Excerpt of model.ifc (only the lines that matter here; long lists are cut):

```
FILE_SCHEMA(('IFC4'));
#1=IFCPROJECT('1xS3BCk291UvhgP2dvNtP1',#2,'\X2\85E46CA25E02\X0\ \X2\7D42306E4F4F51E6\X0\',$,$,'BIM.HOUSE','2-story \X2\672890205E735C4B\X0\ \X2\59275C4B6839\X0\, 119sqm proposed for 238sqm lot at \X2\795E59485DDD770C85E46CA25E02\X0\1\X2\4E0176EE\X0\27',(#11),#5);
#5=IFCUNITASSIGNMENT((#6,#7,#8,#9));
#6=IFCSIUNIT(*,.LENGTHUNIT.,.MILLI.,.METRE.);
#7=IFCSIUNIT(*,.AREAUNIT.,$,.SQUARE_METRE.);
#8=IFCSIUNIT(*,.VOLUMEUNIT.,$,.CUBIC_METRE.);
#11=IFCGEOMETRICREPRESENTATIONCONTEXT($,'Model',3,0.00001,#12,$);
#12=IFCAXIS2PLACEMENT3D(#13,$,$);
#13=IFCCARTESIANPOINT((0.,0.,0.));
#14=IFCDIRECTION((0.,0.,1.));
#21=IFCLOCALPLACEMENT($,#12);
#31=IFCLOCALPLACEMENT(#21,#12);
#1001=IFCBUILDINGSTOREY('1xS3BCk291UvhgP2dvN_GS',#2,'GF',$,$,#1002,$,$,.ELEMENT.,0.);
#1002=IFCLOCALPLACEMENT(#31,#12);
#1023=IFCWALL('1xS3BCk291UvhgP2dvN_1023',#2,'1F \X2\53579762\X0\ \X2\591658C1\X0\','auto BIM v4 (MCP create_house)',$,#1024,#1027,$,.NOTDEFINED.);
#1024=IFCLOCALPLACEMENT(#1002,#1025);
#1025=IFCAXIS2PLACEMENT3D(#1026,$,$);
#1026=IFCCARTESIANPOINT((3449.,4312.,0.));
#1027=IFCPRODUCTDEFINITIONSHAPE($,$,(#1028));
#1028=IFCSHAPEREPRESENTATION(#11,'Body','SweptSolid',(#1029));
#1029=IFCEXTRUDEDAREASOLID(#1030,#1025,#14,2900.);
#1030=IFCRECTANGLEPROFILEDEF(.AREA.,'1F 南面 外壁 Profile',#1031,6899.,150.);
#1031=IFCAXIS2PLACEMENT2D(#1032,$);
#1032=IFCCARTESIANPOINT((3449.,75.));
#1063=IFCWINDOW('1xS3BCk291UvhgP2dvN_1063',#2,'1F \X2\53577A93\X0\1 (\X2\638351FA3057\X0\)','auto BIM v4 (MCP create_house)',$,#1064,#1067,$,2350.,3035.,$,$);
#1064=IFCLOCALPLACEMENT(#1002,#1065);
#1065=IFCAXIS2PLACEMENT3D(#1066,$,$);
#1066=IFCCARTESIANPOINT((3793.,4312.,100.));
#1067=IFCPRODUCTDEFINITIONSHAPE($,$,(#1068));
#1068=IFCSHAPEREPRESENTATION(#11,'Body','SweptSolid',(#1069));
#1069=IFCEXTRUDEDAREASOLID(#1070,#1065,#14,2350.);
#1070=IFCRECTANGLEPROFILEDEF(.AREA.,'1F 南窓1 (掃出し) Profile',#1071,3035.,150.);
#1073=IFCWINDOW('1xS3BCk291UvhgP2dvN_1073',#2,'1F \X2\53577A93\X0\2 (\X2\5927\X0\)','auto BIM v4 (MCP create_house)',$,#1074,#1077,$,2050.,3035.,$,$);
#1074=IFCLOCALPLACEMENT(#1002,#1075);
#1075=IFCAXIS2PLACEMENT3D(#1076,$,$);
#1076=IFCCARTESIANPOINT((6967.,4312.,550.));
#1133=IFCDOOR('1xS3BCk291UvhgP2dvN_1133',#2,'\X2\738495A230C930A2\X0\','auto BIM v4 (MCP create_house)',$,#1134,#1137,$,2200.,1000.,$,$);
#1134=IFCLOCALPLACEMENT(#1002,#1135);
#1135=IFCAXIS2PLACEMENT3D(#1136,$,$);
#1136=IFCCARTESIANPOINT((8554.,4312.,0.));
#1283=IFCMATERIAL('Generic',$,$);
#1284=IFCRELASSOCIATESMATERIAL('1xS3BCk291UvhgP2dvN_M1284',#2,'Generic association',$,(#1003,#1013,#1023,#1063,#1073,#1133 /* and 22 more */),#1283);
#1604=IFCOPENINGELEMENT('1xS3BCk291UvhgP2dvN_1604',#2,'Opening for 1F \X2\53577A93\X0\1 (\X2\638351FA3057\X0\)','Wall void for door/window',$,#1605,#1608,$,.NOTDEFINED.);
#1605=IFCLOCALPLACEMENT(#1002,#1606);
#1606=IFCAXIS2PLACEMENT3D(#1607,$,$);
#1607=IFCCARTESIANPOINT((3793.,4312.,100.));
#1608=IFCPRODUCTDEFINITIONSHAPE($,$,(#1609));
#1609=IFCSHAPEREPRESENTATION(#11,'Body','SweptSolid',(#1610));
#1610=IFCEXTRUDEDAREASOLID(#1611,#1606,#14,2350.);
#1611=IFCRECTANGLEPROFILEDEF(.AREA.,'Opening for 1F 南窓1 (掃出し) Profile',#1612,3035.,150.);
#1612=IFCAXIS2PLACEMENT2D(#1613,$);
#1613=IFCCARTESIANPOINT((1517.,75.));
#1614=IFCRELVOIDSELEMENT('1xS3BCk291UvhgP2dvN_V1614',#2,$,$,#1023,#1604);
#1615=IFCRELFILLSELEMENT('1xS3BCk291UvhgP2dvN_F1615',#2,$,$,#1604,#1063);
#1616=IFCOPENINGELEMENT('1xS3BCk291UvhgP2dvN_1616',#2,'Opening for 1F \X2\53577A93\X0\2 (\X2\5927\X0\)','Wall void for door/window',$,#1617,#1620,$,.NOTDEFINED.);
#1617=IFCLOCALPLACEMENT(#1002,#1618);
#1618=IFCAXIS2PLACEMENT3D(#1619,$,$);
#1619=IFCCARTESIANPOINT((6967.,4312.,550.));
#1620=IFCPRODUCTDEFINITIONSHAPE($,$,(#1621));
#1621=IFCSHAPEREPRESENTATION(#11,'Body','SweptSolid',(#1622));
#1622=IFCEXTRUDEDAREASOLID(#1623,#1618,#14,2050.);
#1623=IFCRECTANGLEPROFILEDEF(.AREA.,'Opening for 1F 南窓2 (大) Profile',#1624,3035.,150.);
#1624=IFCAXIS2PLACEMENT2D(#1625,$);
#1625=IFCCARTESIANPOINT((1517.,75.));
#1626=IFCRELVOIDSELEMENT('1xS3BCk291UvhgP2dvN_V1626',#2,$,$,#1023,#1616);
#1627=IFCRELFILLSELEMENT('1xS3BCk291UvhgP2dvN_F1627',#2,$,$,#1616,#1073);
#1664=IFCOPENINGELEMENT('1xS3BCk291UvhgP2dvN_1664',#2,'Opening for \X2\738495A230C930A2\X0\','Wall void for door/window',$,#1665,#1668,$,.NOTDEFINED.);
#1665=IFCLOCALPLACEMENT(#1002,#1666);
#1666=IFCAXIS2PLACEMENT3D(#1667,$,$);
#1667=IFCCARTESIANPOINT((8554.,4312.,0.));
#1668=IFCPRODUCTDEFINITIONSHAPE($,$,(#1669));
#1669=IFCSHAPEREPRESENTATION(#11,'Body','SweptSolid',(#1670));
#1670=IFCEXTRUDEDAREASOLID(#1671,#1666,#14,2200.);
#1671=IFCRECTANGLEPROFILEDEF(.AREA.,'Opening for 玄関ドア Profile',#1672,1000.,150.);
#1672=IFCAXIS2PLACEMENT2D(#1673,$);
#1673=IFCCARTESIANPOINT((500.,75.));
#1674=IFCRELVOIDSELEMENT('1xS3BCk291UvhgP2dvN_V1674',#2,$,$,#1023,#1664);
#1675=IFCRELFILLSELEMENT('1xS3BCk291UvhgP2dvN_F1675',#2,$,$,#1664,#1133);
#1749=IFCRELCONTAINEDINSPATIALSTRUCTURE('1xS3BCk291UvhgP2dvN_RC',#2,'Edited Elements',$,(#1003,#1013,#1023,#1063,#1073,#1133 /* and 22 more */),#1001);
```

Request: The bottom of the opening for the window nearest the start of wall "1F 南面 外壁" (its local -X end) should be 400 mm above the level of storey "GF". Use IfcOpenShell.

```python
import numpy as np
import ifcopenshell
import ifcopenshell.api.geometry
import ifcopenshell.geom
import ifcopenshell.util.element
import ifcopenshell.util.placement
import ifcopenshell.util.shape
import ifcopenshell.util.unit

model = ifcopenshell.open("model.ifc")
unit_scale = ifcopenshell.util.unit.calculate_unit_scale(model)

window = model.by_id(1063)
opening = window.FillsVoids[0].RelatingOpeningElement
storey = ifcopenshell.util.element.get_container(window, ifc_class="IfcBuildingStorey")
level = ifcopenshell.util.placement.get_local_placement(storey.ObjectPlacement)[2, 3]

# The opening's origin need not be at the sill, so measure its lowest point.
shape = ifcopenshell.geom.create_shape(ifcopenshell.geom.settings(), opening)
bottom = ifcopenshell.util.shape.get_shape_bottom_elevation(shape, shape.geometry) / unit_scale
dz = level + 400.0 - bottom

shift = np.array([0.0, 0.0, dz])
# The window is not placed relative to its opening, so move both.
for product in (opening, window):
    matrix = ifcopenshell.util.placement.get_local_placement(product.ObjectPlacement)
    matrix[:3, 3] += shift
    ifcopenshell.api.geometry.edit_object_placement(model, product=product, matrix=matrix, is_si=False)

print(f"moved by {dz * unit_scale:+.3f} m")

model.write("model_v2.ifc")
```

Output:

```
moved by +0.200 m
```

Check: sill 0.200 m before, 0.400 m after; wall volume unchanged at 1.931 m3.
